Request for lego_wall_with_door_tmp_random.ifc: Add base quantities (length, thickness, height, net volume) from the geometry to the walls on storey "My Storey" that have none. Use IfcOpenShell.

First a look at what the model holds.

```python
import ifcopenshell
import ifcopenshell.util.element
import ifcopenshell.util.unit

model = ifcopenshell.open("lego_wall_with_door_tmp_random.ifc")
print(model.schema)
for unit_type in ("LENGTHUNIT", "AREAUNIT", "VOLUMEUNIT"):
    print(unit_type, ifcopenshell.util.unit.calculate_unit_scale(model, unit_type))
storey = next(s for s in model.by_type("IfcBuildingStorey") if s.Name == "My Storey")
walls = [e for e in ifcopenshell.util.element.get_decomposition(storey) if e.is_a("IfcWall")]
for e in sorted(walls, key=lambda e: e.id()):
    print(e.id(), e.is_a(), e.Name, list(ifcopenshell.util.element.get_psets(e, qtos_only=True)), sep=" | ")
```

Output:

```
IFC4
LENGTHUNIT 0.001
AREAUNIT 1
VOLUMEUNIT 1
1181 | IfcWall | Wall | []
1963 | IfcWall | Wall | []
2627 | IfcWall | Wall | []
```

```python
import ifcopenshell
import ifcopenshell.api.pset
import ifcopenshell.geom
import ifcopenshell.util.element
import ifcopenshell.util.shape
import ifcopenshell.util.unit

model = ifcopenshell.open("lego_wall_with_door_tmp_random.ifc")
unit_scale = ifcopenshell.util.unit.calculate_unit_scale(model)
volume_scale = ifcopenshell.util.unit.calculate_unit_scale(model, "VOLUMEUNIT")
settings = ifcopenshell.geom.settings()

storey = next(s for s in model.by_type("IfcBuildingStorey") if s.Name == "My Storey")
walls = [e for e in ifcopenshell.util.element.get_decomposition(storey) if e.is_a("IfcWall")]

for e in sorted(walls, key=lambda e: e.id()):
    if ifcopenshell.util.element.get_psets(e, qtos_only=True, should_inherit=False):
        continue
    # Geometry comes back in metres, in the element's own axes.
    shape = ifcopenshell.geom.create_shape(settings, e)
    values = {
        "Length": ifcopenshell.util.shape.get_x(shape.geometry) / unit_scale,
        "Width": ifcopenshell.util.shape.get_y(shape.geometry) / unit_scale,
        "Height": ifcopenshell.util.shape.get_z(shape.geometry) / unit_scale,
        "NetVolume": ifcopenshell.util.shape.get_volume(shape.geometry) / volume_scale,
    }
    qto = ifcopenshell.api.pset.add_qto(model, product=e, name="Qto_WallBaseQuantities")
    ifcopenshell.api.pset.edit_qto(model, qto=qto, properties=values)
    print(e.id(), {k: round(v, 3) for k, v in values.items()})

model.write("lego_wall_with_door_tmp_random-out.ifc")
```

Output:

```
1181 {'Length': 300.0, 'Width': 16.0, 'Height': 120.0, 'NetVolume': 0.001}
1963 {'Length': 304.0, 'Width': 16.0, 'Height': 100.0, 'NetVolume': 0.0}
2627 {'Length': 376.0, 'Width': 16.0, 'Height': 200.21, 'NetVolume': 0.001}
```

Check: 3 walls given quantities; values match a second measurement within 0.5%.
